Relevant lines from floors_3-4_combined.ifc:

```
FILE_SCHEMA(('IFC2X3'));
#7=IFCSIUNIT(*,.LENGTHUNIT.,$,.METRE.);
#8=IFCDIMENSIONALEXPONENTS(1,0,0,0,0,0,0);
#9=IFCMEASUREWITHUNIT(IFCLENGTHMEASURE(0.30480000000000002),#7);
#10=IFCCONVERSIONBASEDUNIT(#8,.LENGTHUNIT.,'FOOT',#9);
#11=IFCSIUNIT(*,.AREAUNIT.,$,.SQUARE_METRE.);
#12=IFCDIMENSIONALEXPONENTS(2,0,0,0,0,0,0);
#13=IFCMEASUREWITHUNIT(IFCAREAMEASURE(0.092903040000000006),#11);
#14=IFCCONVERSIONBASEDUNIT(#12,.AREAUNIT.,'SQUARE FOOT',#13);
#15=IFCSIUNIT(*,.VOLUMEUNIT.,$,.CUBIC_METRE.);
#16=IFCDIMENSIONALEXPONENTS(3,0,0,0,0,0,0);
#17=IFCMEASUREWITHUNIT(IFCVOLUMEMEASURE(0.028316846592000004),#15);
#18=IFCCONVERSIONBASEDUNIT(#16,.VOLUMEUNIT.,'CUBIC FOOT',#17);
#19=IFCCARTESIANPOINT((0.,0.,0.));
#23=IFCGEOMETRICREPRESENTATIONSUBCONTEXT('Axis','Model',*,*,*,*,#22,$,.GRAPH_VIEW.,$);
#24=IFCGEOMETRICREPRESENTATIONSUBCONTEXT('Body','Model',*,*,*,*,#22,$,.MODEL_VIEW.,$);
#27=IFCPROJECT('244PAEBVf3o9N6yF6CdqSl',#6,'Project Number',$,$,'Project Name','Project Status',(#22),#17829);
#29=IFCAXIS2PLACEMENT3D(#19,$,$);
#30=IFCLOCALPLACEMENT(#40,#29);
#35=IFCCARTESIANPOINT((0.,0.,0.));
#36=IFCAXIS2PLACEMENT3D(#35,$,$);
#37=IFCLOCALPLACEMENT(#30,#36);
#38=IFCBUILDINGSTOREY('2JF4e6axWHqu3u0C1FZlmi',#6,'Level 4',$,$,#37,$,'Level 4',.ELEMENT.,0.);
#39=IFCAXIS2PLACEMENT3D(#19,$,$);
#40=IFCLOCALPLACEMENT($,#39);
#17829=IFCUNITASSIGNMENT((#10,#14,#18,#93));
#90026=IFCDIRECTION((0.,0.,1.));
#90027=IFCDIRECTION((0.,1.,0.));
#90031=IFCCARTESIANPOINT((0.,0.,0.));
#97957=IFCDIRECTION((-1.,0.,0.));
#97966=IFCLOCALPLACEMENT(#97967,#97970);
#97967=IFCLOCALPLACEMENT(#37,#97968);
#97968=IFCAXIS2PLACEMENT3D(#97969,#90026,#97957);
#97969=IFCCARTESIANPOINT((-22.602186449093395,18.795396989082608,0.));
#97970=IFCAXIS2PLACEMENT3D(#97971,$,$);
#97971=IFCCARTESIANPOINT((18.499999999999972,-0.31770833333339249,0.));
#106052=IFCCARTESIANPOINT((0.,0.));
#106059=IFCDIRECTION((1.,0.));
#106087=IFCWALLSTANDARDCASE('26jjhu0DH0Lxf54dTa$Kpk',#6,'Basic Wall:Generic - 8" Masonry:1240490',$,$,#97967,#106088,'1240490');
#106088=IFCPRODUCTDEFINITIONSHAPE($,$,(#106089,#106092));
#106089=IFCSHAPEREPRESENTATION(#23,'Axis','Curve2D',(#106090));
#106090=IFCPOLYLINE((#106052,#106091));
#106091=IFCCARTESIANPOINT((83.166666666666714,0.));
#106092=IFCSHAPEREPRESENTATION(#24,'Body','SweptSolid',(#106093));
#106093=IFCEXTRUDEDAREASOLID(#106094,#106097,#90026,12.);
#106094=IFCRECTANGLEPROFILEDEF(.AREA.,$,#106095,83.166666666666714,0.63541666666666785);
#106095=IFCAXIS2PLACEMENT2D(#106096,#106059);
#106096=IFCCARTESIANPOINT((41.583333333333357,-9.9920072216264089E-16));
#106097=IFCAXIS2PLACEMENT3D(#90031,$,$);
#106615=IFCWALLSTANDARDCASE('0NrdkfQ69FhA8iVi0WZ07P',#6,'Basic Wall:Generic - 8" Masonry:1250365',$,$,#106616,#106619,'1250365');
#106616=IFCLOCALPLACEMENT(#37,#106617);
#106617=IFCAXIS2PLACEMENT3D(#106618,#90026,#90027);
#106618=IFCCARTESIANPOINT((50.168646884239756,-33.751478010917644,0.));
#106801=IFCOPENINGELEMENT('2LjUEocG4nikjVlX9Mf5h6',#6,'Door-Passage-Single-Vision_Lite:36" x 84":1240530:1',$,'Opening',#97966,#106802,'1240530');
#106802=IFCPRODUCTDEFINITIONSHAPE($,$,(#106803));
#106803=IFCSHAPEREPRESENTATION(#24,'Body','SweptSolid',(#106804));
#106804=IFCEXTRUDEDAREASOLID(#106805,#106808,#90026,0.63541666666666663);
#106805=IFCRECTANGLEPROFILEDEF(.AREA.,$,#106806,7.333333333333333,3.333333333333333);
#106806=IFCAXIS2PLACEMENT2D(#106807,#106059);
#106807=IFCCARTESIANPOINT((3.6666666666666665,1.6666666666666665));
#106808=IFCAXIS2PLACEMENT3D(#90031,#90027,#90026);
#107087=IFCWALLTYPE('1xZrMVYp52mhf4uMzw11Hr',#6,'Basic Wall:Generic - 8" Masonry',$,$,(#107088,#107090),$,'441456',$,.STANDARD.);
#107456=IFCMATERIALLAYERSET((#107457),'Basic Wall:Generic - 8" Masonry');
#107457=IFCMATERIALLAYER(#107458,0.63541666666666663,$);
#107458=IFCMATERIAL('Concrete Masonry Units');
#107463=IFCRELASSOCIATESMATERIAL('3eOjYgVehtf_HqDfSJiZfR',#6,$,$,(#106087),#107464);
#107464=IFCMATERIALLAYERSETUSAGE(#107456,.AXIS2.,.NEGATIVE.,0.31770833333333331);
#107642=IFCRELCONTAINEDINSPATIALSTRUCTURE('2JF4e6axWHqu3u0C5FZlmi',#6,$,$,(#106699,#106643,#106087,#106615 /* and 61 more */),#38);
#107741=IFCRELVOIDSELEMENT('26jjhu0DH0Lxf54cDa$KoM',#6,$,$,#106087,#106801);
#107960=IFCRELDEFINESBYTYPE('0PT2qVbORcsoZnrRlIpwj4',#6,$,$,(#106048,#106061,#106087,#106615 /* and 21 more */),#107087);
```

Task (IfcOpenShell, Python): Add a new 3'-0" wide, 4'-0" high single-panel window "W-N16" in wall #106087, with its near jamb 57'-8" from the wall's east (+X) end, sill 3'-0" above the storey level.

```python
import numpy as np
import ifcopenshell
import ifcopenshell.api.feature
import ifcopenshell.api.geometry
import ifcopenshell.api.root
import ifcopenshell.api.spatial
import ifcopenshell.api.type
import ifcopenshell.geom
import ifcopenshell.util.element
import ifcopenshell.util.placement
import ifcopenshell.util.representation
import ifcopenshell.util.shape
import ifcopenshell.util.unit

model = ifcopenshell.open("floors_3-4_combined.ifc")
unit_scale = ifcopenshell.util.unit.calculate_unit_scale(model)
settings = ifcopenshell.geom.settings()


def volume(element):
    """Net volume in cubic metres, openings subtracted."""
    shape = ifcopenshell.geom.create_shape(settings, element)
    return ifcopenshell.util.shape.get_volume(shape.geometry)


wall = model.by_guid("26jjhu0DH0Lxf54dTa$Kpk")
storey = ifcopenshell.util.element.get_container(wall, ifc_class="IfcBuildingStorey")
context = ifcopenshell.util.representation.get_context(model, "Model", "Body", "MODEL_VIEW")
before = volume(wall)

width, height, from_end, sill = 0.9144, 1.2192, 17.5768, 0.9144  # metres

# The wall runs along its own X axis, and the end named is its -X end.
wall_shape = ifcopenshell.geom.create_shape(settings, wall)
x, y, z = ifcopenshell.util.shape.get_vertices(wall_shape.geometry).T
start = x.min() + from_end
face, thickness = float(y.min()), float(y.max() - y.min())
wall_matrix = ifcopenshell.util.placement.get_local_placement(wall.ObjectPlacement)
level = ifcopenshell.util.placement.get_local_placement(storey.ObjectPlacement)[2, 3]


def in_wall(x, y):
    """Placement at x, y metres in the wall's axes, at sill height."""
    matrix = wall_matrix.copy()
    matrix[:, 3] = wall_matrix @ np.array([x / unit_scale, y / unit_scale, 0.0, 1.0])
    matrix[2, 3] = level + sill / unit_scale
    return matrix


# Opening: a box that overshoots both wall faces by 50 mm.
opening = ifcopenshell.api.root.create_entity(model, ifc_class="IfcOpeningElement")
box = ifcopenshell.api.geometry.add_wall_representation(
    model, context=context, length=width, height=height, thickness=thickness + 0.1
)
ifcopenshell.api.geometry.assign_representation(model, product=opening, representation=box)
ifcopenshell.api.geometry.edit_object_placement(model, product=opening, matrix=in_wall(start, face - 0.05), is_si=False)
ifcopenshell.api.feature.add_feature(model, feature=opening, element=wall)

window = ifcopenshell.api.root.create_entity(model, ifc_class="IfcWindow", name="W-N16")
window.OverallWidth, window.OverallHeight = width / unit_scale, height / unit_scale
body = ifcopenshell.api.geometry.add_window_representation(
    model,
    context=context,
    overall_width=window.OverallWidth,
    overall_height=window.OverallHeight,
    partition_type="SINGLE_PANEL",
)
ifcopenshell.api.geometry.assign_representation(model, product=window, representation=body)
ifcopenshell.api.spatial.assign_container(model, products=[window], relating_structure=storey)
fills = ifcopenshell.api.feature.add_filling(model, opening=opening, element=window)
fills.OwnerHistory = window.OwnerHistory  # required in IFC2X3

# IFC2X3 keeps the operation on the window style.
style = ifcopenshell.api.root.create_entity(model, ifc_class="IfcWindowStyle", name="W-N16")
style.OperationType, style.ConstructionType = "SINGLE_PANEL", "NOTDEFINED"
style.ParameterTakesPrecedence = style.Sizeable = False
ifcopenshell.api.type.assign_type(model, related_objects=[window], relating_type=style)

# Centre the window in the wall's thickness.
ifcopenshell.api.geometry.edit_object_placement(model, product=window, matrix=in_wall(start, face), is_si=False)
window_shape = ifcopenshell.geom.create_shape(settings, window)
depth = ifcopenshell.util.shape.get_vertices(window_shape.geometry)[:, 1]
offset = face + thickness / 2 - (depth.min() + depth.max()) / 2
ifcopenshell.api.geometry.edit_object_placement(model, product=window, matrix=in_wall(start, offset), is_si=False)

after = volume(wall)

print(f"wall volume {before:.3f} -> {after:.3f} m3")

model.write("floors_3-4_combined_edited.ifc")
```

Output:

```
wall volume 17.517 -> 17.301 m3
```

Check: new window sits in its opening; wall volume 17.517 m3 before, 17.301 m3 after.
